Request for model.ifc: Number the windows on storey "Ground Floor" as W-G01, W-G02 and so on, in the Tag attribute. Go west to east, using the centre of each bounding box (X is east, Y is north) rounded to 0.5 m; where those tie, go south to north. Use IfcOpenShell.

First a look at what the model holds.

```python
import ifcopenshell
import ifcopenshell.util.element
import ifcopenshell.util.placement

model = ifcopenshell.open("model.ifc")
print(model.schema)
storey = next(s for s in model.by_type("IfcBuildingStorey") if s.Name == "Ground Floor")
windows = [e for e in ifcopenshell.util.element.get_decomposition(storey) if e.is_a("IfcWindow")]
for e in sorted(windows, key=lambda e: e.id()):
    origin = ifcopenshell.util.placement.get_local_placement(e.ObjectPlacement)[:3, 3]
    print(e.id(), e.Tag, e.Name, origin.round(2) + 0.0, sep=" | ")
```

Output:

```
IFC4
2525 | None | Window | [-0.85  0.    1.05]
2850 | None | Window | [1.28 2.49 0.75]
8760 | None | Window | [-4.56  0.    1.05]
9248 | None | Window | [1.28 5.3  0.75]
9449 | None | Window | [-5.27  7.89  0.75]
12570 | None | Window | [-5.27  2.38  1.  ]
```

```python
import ifcopenshell
import ifcopenshell.geom
import ifcopenshell.util.element
import ifcopenshell.util.shape

model = ifcopenshell.open("model.ifc")
settings = ifcopenshell.geom.settings()
settings.set("use-world-coords", True)


def centre(element):
    shape = ifcopenshell.geom.create_shape(settings, element)
    return ifcopenshell.util.shape.get_bbox_centroid(shape.geometry)


storey = next(s for s in model.by_type("IfcBuildingStorey") if s.Name == "Ground Floor")
windows = [e for e in ifcopenshell.util.element.get_decomposition(storey) if e.is_a("IfcWindow")]

# Insertion points can sit at a corner or the storey origin, so sort by the geometry (in metres).
centres = {e: centre(e) for e in windows}
windows.sort(key=lambda e: (round(centres[e][0] / 0.5), centres[e][1]))

for i, e in enumerate(windows, start=1):
    number = f"W-G{i:02d}"
    e.Tag = number
    print(e.id(), number)

model.write("model_updated.ifc")
```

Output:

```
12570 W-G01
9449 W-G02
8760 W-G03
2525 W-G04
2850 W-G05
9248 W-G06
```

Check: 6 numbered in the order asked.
